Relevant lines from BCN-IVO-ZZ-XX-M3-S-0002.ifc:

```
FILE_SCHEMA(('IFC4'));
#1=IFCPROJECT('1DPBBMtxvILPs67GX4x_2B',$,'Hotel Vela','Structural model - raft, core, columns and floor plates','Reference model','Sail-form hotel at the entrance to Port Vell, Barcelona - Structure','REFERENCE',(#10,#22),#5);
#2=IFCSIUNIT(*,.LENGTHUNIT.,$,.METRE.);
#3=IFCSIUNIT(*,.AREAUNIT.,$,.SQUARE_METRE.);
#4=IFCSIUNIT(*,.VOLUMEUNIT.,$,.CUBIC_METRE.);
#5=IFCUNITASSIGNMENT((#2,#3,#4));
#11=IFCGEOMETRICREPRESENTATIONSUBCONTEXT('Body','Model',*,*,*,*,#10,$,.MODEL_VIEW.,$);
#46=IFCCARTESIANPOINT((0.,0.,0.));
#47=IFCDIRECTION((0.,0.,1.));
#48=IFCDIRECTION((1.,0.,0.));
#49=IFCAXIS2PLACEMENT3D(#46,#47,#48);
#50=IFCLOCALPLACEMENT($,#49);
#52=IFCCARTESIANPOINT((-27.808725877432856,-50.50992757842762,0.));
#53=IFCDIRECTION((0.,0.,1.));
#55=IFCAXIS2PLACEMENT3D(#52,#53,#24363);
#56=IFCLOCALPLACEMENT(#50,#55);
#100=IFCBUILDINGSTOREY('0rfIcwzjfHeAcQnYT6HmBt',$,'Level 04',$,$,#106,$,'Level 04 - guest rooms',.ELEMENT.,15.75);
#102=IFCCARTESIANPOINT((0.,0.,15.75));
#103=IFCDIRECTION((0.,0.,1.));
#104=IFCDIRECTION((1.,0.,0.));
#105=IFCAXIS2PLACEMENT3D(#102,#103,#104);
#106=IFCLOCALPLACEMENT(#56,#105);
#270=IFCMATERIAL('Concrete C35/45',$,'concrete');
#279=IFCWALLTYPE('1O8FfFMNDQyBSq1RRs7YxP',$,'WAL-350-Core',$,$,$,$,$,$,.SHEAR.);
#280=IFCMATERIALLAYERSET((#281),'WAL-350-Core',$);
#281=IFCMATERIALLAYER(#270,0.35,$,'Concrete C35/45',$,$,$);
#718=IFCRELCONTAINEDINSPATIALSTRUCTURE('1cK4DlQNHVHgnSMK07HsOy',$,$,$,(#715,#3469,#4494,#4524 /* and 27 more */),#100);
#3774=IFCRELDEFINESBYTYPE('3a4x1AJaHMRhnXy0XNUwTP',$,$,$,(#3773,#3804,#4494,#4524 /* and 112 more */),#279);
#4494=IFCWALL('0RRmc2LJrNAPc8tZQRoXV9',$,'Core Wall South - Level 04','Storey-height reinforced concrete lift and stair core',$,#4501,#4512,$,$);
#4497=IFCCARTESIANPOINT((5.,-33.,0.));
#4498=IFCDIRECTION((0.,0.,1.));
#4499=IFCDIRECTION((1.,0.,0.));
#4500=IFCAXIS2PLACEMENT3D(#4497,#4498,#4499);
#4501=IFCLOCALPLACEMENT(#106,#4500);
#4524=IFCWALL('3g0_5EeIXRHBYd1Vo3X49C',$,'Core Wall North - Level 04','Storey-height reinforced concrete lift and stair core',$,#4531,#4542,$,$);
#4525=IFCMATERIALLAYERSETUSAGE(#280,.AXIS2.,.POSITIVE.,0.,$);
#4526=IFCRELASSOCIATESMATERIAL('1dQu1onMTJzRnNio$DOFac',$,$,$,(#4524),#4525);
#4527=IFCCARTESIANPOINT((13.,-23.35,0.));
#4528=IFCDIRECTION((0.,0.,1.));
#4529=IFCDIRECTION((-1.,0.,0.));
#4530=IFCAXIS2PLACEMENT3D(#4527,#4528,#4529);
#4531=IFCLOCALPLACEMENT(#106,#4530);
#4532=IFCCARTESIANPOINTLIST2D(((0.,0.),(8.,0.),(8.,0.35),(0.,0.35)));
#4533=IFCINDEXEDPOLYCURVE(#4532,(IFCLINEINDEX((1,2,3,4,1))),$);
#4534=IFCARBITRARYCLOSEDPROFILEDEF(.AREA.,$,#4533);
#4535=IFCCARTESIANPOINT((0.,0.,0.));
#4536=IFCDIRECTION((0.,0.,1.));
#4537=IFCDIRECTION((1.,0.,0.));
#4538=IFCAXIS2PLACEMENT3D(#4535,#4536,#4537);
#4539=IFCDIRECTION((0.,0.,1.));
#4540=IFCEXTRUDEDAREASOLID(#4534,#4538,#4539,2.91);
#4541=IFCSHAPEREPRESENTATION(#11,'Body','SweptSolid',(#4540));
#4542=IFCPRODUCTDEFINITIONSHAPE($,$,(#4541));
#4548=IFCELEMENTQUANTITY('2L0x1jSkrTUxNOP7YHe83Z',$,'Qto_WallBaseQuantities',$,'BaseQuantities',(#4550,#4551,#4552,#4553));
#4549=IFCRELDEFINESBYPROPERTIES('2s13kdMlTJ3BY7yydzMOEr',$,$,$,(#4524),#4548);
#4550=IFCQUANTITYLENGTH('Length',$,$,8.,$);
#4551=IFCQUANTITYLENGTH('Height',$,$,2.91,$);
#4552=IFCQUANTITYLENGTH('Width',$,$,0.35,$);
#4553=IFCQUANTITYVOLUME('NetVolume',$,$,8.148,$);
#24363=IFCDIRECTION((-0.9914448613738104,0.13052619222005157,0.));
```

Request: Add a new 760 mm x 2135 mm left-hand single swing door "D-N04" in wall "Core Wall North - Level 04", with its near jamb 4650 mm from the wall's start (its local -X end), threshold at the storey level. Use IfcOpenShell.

```python
import numpy as np
import ifcopenshell
import ifcopenshell.api.feature
import ifcopenshell.api.geometry
import ifcopenshell.api.pset
import ifcopenshell.api.root
import ifcopenshell.api.spatial
import ifcopenshell.geom
import ifcopenshell.util.element
import ifcopenshell.util.placement
import ifcopenshell.util.representation
import ifcopenshell.util.shape
import ifcopenshell.util.unit

model = ifcopenshell.open("BCN-IVO-ZZ-XX-M3-S-0002.ifc")
unit_scale = ifcopenshell.util.unit.calculate_unit_scale(model)
volume_scale = ifcopenshell.util.unit.calculate_unit_scale(model, "VOLUMEUNIT")
settings = ifcopenshell.geom.settings()


def volume(element):
    """Net volume in cubic metres, openings subtracted."""
    shape = ifcopenshell.geom.create_shape(settings, element)
    return ifcopenshell.util.shape.get_volume(shape.geometry)


wall = model.by_guid("3g0_5EeIXRHBYd1Vo3X49C")
storey = ifcopenshell.util.element.get_container(wall, ifc_class="IfcBuildingStorey")
context = ifcopenshell.util.representation.get_context(model, "Model", "Body", "MODEL_VIEW")
before = volume(wall)

width, height, from_end, sill = 0.76, 2.135, 4.65, 0.0  # metres

# The wall runs along its own X axis, and the end named is its -X end.
wall_shape = ifcopenshell.geom.create_shape(settings, wall)
x, y, z = ifcopenshell.util.shape.get_vertices(wall_shape.geometry).T
start = x.min() + from_end
face, thickness = float(y.min()), float(y.max() - y.min())
wall_matrix = ifcopenshell.util.placement.get_local_placement(wall.ObjectPlacement)
level = ifcopenshell.util.placement.get_local_placement(storey.ObjectPlacement)[2, 3]


def in_wall(x, y):
    """Placement at x, y metres in the wall's axes, at sill height."""
    matrix = wall_matrix.copy()
    matrix[:, 3] = wall_matrix @ np.array([x / unit_scale, y / unit_scale, 0.0, 1.0])
    matrix[2, 3] = level + sill / unit_scale
    return matrix


# Opening: a box that overshoots both wall faces by 50 mm.
opening = ifcopenshell.api.root.create_entity(model, ifc_class="IfcOpeningElement", predefined_type="OPENING")
box = ifcopenshell.api.geometry.add_wall_representation(
    model, context=context, length=width, height=height, thickness=thickness + 0.1
)
ifcopenshell.api.geometry.assign_representation(model, product=opening, representation=box)
ifcopenshell.api.geometry.edit_object_placement(model, product=opening, matrix=in_wall(start, face - 0.05), is_si=False)
ifcopenshell.api.feature.add_feature(model, feature=opening, element=wall)

door = ifcopenshell.api.root.create_entity(model, ifc_class="IfcDoor", name="D-N04", predefined_type="DOOR")
door.OverallWidth, door.OverallHeight = width / unit_scale, height / unit_scale
door.OperationType = "SINGLE_SWING_LEFT"
body = ifcopenshell.api.geometry.add_door_representation(
    model,
    context=context,
    overall_width=door.OverallWidth,
    overall_height=door.OverallHeight,
    operation_type="SINGLE_SWING_LEFT",
    lining_properties={"LiningDepth": thickness / unit_scale, "ThresholdDepth": thickness / unit_scale},
)
ifcopenshell.api.geometry.assign_representation(model, product=door, representation=body)
ifcopenshell.api.spatial.assign_container(model, products=[door], relating_structure=storey)
ifcopenshell.api.feature.add_filling(model, opening=opening, element=door)

# The lining spans the wall, so the door starts at the wall face.
ifcopenshell.api.geometry.edit_object_placement(model, product=door, matrix=in_wall(start, face), is_si=False)

after = volume(wall)

# Update the wall's stored quantities.
qto = model.by_id(ifcopenshell.util.element.get_pset(wall, "Qto_WallBaseQuantities", should_inherit=False)["id"])
ifcopenshell.api.pset.edit_qto(model, qto=qto, properties={"NetVolume": after / volume_scale})

print(f"wall volume {before:.3f} -> {after:.3f} m3")

model.write("BCN-IVO-ZZ-XX-M3-S-0002_updated.ifc")
```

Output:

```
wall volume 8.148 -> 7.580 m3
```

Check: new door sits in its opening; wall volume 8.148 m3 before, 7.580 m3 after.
